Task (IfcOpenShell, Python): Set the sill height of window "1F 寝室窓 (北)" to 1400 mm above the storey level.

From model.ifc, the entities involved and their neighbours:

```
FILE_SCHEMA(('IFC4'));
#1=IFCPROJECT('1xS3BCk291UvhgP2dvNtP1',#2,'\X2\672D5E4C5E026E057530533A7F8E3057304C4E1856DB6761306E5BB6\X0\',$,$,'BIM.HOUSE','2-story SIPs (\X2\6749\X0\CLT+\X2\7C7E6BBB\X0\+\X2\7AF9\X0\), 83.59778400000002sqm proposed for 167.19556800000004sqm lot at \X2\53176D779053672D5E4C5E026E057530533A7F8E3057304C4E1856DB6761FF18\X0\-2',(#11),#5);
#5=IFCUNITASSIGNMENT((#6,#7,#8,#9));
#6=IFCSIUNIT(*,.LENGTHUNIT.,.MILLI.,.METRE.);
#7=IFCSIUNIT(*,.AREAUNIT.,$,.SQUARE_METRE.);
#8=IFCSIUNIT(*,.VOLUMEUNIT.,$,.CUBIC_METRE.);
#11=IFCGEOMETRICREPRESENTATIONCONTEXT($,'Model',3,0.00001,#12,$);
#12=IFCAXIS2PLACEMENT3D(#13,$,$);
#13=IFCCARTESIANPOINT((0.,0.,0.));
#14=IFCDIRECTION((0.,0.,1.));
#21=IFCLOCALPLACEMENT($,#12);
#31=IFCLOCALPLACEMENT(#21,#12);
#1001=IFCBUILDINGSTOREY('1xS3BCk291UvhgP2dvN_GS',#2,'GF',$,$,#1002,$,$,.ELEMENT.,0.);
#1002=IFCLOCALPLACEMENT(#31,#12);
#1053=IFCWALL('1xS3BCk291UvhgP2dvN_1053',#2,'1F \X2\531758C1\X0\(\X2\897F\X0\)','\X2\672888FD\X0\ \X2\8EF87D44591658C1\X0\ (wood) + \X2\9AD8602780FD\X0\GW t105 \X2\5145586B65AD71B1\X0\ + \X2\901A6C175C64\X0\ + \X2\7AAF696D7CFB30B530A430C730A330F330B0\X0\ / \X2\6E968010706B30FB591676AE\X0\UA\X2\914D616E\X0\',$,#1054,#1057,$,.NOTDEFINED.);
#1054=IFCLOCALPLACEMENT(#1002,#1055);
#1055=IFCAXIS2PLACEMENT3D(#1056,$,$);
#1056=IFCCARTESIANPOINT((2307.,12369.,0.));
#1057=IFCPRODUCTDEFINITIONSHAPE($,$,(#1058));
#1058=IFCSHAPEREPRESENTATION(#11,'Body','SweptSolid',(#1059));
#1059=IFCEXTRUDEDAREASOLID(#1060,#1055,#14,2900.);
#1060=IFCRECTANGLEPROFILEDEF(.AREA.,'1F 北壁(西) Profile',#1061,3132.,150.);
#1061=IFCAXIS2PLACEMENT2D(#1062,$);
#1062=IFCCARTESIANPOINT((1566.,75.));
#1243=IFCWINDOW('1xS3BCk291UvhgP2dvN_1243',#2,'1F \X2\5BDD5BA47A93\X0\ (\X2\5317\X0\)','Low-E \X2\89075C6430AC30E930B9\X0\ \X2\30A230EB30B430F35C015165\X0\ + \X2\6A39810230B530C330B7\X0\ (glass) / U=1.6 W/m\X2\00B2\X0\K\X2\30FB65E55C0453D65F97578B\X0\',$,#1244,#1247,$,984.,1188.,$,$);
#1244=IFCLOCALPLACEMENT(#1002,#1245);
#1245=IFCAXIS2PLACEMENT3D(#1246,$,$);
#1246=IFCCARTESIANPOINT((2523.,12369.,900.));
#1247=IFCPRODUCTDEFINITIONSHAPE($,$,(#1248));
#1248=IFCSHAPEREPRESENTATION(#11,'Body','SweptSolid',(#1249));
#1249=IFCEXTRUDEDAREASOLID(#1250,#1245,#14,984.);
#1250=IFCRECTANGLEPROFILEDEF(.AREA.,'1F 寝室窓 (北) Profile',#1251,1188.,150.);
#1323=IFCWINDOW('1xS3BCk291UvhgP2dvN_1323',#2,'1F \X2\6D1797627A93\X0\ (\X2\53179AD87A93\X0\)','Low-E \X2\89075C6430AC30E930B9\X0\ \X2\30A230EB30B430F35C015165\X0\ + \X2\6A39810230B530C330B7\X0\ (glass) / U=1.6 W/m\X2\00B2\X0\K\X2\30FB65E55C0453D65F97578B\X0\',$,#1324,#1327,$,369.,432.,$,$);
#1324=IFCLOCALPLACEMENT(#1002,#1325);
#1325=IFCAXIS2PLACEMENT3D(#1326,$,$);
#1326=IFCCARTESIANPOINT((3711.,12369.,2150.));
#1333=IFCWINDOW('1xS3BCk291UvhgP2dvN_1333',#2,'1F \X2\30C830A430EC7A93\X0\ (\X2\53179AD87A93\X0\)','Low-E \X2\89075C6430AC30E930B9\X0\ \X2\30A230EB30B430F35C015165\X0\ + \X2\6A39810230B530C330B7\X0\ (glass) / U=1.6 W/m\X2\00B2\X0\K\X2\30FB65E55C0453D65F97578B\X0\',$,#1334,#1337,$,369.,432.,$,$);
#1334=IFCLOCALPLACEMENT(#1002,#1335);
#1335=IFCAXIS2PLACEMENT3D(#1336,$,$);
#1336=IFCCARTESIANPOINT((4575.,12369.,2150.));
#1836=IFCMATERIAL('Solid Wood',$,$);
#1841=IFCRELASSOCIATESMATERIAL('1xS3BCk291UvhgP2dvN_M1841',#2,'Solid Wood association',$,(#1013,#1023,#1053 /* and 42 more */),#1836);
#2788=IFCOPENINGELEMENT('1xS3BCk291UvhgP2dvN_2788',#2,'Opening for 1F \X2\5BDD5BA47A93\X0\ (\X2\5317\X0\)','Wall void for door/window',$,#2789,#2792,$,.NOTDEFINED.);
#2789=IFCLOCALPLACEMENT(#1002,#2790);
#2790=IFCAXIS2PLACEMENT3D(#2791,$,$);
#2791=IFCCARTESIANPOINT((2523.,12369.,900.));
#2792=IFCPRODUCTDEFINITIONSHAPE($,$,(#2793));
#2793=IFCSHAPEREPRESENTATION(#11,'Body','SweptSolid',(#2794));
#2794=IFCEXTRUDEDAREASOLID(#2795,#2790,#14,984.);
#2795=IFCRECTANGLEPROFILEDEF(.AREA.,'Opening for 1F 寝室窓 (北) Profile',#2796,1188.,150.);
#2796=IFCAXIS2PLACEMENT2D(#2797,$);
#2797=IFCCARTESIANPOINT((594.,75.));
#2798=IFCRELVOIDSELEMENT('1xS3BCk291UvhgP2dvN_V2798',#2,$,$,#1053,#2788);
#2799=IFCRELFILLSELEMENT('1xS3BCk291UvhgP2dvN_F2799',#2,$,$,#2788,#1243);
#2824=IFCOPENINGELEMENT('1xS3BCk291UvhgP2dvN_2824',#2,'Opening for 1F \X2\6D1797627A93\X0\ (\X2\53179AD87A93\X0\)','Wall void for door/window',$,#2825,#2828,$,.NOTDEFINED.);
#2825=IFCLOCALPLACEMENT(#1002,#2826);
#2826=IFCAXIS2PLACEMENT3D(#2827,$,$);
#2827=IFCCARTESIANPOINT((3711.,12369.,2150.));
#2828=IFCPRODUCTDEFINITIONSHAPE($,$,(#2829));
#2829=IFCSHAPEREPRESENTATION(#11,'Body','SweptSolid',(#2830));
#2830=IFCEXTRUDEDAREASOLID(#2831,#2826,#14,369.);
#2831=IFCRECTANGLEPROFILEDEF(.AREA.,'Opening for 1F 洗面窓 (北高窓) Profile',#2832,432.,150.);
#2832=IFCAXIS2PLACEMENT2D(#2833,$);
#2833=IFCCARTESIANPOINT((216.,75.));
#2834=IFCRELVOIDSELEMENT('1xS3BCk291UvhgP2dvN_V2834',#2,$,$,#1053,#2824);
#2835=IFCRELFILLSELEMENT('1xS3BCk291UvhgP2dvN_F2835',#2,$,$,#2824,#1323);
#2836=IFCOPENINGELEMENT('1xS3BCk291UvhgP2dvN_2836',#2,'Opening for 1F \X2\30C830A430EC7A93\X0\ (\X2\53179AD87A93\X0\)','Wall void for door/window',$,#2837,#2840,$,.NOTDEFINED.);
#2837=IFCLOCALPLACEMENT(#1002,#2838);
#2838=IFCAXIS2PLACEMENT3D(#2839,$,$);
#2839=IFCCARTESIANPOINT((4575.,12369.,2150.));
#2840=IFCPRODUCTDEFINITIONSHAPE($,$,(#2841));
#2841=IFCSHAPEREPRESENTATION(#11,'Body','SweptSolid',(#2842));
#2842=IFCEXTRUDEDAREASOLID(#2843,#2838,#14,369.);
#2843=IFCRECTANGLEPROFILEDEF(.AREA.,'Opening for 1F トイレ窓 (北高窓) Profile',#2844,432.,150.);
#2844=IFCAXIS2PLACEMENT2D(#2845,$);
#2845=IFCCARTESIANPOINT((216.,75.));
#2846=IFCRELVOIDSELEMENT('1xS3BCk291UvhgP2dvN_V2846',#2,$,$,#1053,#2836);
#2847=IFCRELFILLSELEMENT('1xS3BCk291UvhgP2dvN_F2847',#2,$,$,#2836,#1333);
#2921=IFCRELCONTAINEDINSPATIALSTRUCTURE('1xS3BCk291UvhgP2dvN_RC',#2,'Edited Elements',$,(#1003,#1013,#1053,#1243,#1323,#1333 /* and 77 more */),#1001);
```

```python
import numpy as np
import ifcopenshell
import ifcopenshell.api.geometry
import ifcopenshell.geom
import ifcopenshell.util.element
import ifcopenshell.util.placement
import ifcopenshell.util.shape
import ifcopenshell.util.unit

model = ifcopenshell.open("model.ifc")
unit_scale = ifcopenshell.util.unit.calculate_unit_scale(model)

window = model.by_guid("1xS3BCk291UvhgP2dvN_1243")
opening = window.FillsVoids[0].RelatingOpeningElement
storey = ifcopenshell.util.element.get_container(window, ifc_class="IfcBuildingStorey")
level = ifcopenshell.util.placement.get_local_placement(storey.ObjectPlacement)[2, 3]

# The opening's origin need not be at the sill, so measure its lowest point.
shape = ifcopenshell.geom.create_shape(ifcopenshell.geom.settings(), opening)
bottom = ifcopenshell.util.shape.get_shape_bottom_elevation(shape, shape.geometry) / unit_scale
dz = level + 1.4 / unit_scale - bottom

shift = np.array([0.0, 0.0, dz])
# The window is not placed relative to its opening, so move both.
for product in (opening, window):
    matrix = ifcopenshell.util.placement.get_local_placement(product.ObjectPlacement)
    matrix[:3, 3] += shift
    ifcopenshell.api.geometry.edit_object_placement(model, product=product, matrix=matrix, is_si=False)

print(f"moved by {dz * unit_scale:+.3f} m")

model.write("model_updated.ifc")
```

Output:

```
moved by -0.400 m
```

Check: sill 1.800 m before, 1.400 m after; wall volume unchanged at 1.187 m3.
